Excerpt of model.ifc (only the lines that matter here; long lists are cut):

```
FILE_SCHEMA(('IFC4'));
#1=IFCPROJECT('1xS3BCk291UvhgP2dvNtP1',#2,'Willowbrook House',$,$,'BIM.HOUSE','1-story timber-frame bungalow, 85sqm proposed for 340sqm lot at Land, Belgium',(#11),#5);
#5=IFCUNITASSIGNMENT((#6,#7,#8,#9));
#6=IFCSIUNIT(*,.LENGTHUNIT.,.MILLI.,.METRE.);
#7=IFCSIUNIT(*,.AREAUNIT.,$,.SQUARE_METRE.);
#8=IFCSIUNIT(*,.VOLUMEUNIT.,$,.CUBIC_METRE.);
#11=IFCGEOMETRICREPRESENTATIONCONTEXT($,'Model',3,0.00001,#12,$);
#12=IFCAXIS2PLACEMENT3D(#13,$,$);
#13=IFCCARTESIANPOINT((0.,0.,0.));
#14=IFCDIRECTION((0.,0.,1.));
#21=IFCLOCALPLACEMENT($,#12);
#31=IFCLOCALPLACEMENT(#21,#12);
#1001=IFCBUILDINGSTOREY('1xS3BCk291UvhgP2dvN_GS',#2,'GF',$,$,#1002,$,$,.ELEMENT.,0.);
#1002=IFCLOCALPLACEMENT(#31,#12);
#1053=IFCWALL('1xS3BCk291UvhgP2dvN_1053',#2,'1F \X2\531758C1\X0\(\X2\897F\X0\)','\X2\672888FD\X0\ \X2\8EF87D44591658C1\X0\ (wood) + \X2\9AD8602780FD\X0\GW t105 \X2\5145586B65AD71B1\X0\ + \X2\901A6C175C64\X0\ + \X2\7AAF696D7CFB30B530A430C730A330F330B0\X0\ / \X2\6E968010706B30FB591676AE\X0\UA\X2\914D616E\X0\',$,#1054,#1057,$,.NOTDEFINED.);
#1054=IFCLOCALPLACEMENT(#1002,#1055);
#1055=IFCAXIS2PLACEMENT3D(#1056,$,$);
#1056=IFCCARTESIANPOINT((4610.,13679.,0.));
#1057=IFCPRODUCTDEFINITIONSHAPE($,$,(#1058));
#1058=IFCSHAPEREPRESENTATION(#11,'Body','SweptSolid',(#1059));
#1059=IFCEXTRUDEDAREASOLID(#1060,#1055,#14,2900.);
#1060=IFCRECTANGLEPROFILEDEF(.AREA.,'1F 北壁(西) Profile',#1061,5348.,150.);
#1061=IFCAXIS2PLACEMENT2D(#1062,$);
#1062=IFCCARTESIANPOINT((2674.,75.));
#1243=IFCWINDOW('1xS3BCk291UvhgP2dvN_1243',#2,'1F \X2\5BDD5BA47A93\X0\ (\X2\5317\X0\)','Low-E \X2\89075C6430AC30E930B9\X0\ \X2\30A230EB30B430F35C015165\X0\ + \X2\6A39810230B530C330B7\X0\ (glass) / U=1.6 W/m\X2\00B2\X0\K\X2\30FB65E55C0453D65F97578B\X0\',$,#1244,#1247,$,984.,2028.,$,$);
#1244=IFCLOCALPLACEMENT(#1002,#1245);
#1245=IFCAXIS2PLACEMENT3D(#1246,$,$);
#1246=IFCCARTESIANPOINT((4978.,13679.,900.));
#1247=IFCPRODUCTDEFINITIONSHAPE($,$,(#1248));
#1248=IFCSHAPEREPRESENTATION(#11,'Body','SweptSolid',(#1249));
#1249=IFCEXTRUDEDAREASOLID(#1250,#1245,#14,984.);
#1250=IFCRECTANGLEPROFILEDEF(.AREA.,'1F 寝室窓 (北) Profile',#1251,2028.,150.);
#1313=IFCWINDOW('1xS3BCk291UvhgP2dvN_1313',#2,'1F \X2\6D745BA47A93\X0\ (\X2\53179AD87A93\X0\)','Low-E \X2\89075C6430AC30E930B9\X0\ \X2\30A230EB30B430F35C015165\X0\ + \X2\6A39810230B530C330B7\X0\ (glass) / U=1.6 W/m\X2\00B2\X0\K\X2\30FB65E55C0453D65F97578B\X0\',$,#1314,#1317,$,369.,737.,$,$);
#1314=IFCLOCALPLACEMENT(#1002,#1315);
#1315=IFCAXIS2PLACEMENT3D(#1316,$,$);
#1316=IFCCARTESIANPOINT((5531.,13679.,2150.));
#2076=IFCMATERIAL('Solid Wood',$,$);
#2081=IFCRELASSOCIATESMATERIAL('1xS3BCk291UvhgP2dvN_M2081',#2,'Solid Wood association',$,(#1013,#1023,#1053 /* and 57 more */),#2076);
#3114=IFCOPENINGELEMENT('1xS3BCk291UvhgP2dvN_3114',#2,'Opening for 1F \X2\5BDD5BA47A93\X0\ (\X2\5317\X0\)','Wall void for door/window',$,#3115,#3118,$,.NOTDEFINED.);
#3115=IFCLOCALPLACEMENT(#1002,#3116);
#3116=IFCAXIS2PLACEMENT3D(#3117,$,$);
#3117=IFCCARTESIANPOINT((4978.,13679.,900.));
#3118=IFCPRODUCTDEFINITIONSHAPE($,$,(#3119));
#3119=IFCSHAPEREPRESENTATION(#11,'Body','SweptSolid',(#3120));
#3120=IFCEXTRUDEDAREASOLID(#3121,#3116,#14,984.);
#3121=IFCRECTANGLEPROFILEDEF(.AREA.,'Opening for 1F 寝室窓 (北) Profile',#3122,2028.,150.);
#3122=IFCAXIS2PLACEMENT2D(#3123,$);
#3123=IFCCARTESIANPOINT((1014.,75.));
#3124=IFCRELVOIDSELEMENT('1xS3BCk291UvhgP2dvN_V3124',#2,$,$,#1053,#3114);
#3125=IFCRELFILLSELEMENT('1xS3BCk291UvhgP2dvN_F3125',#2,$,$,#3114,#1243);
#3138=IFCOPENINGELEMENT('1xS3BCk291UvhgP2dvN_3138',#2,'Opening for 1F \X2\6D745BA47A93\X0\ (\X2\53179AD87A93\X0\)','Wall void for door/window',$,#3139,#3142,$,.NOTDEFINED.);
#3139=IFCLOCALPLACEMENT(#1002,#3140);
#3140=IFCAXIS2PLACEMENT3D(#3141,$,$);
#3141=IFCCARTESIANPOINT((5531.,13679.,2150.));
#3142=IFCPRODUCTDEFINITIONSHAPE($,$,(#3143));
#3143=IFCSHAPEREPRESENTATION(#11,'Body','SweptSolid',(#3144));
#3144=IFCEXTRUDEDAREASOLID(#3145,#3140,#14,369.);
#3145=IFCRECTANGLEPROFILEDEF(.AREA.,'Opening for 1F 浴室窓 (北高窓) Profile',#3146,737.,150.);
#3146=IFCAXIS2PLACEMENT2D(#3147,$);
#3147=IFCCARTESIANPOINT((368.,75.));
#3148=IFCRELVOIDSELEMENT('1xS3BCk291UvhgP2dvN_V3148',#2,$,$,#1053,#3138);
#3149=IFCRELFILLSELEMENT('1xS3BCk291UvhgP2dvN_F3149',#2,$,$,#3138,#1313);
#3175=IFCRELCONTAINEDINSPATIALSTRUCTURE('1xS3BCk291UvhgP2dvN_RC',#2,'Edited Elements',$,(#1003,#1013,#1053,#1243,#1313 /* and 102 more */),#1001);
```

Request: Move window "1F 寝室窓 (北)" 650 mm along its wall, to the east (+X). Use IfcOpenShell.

```python
import ifcopenshell
import ifcopenshell.api.geometry
import ifcopenshell.util.placement

model = ifcopenshell.open("model.ifc")

window = model.by_guid("1xS3BCk291UvhgP2dvN_1243")
opening = window.FillsVoids[0].RelatingOpeningElement
wall = opening.VoidsElements[0].RelatingBuildingElement

wall_matrix = ifcopenshell.util.placement.get_local_placement(wall.ObjectPlacement)
shift = wall_matrix[:3, 0] * 650.0
before = ifcopenshell.util.placement.get_local_placement(window.ObjectPlacement)[:3, 3].copy()

# The window is not placed relative to its opening, so move both.
for product in (opening, window):
    matrix = ifcopenshell.util.placement.get_local_placement(product.ObjectPlacement)
    matrix[:3, 3] += shift
    ifcopenshell.api.geometry.edit_object_placement(model, product=product, matrix=matrix, is_si=False)

after = ifcopenshell.util.placement.get_local_placement(window.ObjectPlacement)[:3, 3]
print("window moved by", (after - before).round(3) + 0.0)

model.write("model_v2.ifc")
```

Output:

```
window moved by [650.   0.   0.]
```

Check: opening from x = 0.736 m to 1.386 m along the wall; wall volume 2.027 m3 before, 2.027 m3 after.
